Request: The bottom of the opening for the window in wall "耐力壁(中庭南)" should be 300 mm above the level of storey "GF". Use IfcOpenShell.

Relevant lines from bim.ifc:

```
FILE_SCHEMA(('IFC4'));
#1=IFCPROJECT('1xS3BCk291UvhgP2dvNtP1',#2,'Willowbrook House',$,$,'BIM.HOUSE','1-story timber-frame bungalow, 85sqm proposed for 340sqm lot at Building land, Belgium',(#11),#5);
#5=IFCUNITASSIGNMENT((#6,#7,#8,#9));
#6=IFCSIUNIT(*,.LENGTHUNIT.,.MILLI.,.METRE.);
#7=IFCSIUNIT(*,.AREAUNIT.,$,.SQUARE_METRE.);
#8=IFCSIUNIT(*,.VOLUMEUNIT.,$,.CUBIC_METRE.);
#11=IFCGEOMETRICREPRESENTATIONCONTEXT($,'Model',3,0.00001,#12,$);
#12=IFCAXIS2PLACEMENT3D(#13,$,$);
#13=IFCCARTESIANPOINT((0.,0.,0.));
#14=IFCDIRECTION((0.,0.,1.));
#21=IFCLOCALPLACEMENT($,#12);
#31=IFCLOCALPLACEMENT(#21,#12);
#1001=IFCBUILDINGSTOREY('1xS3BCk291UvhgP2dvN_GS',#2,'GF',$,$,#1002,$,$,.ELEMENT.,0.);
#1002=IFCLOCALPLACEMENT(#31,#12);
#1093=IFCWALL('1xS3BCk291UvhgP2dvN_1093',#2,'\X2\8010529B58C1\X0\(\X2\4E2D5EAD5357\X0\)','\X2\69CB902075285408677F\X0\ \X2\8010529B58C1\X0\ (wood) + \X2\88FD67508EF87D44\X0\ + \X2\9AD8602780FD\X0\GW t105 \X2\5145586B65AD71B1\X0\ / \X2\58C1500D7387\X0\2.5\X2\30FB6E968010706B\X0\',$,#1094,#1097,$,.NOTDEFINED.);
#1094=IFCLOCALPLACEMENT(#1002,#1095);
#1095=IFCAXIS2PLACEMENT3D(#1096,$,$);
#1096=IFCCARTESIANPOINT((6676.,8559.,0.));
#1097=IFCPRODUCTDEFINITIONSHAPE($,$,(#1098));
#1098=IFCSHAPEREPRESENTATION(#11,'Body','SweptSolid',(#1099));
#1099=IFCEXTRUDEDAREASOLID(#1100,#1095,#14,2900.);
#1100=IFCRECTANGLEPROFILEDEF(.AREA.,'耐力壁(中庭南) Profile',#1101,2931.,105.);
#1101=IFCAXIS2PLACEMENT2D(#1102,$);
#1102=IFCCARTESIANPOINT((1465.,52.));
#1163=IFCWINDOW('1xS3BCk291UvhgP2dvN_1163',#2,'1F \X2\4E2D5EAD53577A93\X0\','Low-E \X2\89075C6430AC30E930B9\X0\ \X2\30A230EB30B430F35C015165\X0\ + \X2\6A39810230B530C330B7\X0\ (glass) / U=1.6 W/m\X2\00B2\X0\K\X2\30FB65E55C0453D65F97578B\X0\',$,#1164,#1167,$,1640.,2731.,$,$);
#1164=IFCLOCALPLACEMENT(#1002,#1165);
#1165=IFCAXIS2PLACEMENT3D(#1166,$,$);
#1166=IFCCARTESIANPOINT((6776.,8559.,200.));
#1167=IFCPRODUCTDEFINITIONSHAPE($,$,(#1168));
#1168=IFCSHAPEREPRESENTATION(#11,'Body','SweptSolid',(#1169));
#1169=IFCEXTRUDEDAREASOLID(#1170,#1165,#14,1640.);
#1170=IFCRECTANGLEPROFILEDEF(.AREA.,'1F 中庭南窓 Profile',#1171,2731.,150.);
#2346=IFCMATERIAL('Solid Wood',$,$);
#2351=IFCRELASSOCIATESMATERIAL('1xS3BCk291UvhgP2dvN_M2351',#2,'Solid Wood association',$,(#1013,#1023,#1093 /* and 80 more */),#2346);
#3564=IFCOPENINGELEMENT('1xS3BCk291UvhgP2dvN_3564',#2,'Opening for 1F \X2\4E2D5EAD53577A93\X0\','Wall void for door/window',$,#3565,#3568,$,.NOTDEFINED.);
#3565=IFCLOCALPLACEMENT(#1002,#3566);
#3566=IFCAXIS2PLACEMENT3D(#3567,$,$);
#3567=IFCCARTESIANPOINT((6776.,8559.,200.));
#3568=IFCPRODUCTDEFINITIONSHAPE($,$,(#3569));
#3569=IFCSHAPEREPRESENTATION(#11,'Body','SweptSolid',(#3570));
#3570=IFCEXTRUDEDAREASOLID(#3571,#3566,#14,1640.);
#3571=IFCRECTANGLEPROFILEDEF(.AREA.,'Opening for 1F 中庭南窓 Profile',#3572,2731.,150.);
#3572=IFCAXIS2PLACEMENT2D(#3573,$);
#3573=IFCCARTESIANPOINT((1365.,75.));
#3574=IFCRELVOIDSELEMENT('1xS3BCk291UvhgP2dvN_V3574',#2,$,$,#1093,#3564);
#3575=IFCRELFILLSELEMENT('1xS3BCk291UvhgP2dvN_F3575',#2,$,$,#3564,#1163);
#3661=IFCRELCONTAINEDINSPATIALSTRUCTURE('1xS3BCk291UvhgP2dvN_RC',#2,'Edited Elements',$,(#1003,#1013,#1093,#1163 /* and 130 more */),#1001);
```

```python
import numpy as np
import ifcopenshell
import ifcopenshell.api.geometry
import ifcopenshell.geom
import ifcopenshell.util.element
import ifcopenshell.util.placement
import ifcopenshell.util.shape
import ifcopenshell.util.unit

model = ifcopenshell.open("bim.ifc")
unit_scale = ifcopenshell.util.unit.calculate_unit_scale(model)

window = model.by_id(1163)
opening = window.FillsVoids[0].RelatingOpeningElement
storey = ifcopenshell.util.element.get_container(window, ifc_class="IfcBuildingStorey")
level = ifcopenshell.util.placement.get_local_placement(storey.ObjectPlacement)[2, 3]

# The opening's origin need not be at the sill, so measure its lowest point.
shape = ifcopenshell.geom.create_shape(ifcopenshell.geom.settings(), opening)
bottom = ifcopenshell.util.shape.get_shape_bottom_elevation(shape, shape.geometry) / unit_scale
dz = level + 0.3 / unit_scale - bottom

shift = np.array([0.0, 0.0, dz])
# The window is not placed relative to its opening, so move both.
for product in (opening, window):
    matrix = ifcopenshell.util.placement.get_local_placement(product.ObjectPlacement)
    matrix[:3, 3] += shift
    ifcopenshell.api.geometry.edit_object_placement(model, product=product, matrix=matrix, is_si=False)

print(f"moved by {dz * unit_scale:+.3f} m")

model.write("bim_edited.ifc")
```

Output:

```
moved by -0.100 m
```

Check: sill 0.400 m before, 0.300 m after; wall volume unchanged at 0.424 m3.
